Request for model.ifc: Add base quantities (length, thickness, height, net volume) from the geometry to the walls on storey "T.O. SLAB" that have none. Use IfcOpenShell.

First a look at what the model holds.

```python
import ifcopenshell
import ifcopenshell.util.element
import ifcopenshell.util.unit

model = ifcopenshell.open("model.ifc")
print(model.schema)
for unit_type in ("LENGTHUNIT", "AREAUNIT", "VOLUMEUNIT"):
    print(unit_type, ifcopenshell.util.unit.calculate_unit_scale(model, unit_type))
storey = next(s for s in model.by_type("IfcBuildingStorey") if s.Name == "T.O. SLAB")
walls = [e for e in ifcopenshell.util.element.get_decomposition(storey) if e.is_a("IfcWall")]
for e in sorted(walls, key=lambda e: e.id()):
    print(e.id(), e.is_a(), e.Name, list(ifcopenshell.util.element.get_psets(e, qtos_only=True)), sep=" | ")
```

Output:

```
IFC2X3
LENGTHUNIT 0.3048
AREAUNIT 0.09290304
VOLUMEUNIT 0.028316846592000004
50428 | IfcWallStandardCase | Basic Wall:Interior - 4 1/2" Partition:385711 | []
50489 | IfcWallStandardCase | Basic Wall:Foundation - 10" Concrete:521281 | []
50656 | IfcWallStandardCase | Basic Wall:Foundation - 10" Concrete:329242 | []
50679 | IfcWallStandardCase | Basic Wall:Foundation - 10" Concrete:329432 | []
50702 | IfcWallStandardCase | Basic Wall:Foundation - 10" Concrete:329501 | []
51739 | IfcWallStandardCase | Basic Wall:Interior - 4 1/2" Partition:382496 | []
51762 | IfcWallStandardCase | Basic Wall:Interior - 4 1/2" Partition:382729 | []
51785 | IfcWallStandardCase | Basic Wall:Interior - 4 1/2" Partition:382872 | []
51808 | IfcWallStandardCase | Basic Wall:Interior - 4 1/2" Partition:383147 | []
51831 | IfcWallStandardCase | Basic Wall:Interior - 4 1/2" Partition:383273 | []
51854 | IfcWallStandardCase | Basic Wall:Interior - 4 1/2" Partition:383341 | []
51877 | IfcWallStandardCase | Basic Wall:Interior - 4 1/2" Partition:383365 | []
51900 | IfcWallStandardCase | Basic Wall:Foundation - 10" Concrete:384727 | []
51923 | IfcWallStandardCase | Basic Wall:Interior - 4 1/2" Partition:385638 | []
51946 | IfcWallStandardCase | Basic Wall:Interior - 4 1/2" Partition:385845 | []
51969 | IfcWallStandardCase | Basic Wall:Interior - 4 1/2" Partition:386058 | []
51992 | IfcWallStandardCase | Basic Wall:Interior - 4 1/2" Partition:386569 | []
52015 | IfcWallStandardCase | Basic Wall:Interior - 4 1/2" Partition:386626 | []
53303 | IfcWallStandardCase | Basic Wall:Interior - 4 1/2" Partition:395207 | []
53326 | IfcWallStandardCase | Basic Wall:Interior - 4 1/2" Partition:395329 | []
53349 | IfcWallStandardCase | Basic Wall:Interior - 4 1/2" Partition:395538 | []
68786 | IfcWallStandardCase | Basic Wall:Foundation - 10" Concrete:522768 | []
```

```python
import ifcopenshell
import ifcopenshell.api.pset
import ifcopenshell.geom
import ifcopenshell.util.element
import ifcopenshell.util.shape
import ifcopenshell.util.unit

model = ifcopenshell.open("model.ifc")
unit_scale = ifcopenshell.util.unit.calculate_unit_scale(model)
volume_scale = ifcopenshell.util.unit.calculate_unit_scale(model, "VOLUMEUNIT")
settings = ifcopenshell.geom.settings()

storey = next(s for s in model.by_type("IfcBuildingStorey") if s.Name == "T.O. SLAB")
walls = [e for e in ifcopenshell.util.element.get_decomposition(storey) if e.is_a("IfcWall")]

for e in sorted(walls, key=lambda e: e.id()):
    if ifcopenshell.util.element.get_psets(e, qtos_only=True, should_inherit=False):
        continue
    # Geometry comes back in metres, in the element's own axes.
    shape = ifcopenshell.geom.create_shape(settings, e)
    values = {
        "Length": ifcopenshell.util.shape.get_x(shape.geometry) / unit_scale,
        "Width": ifcopenshell.util.shape.get_y(shape.geometry) / unit_scale,
        "Height": ifcopenshell.util.shape.get_z(shape.geometry) / unit_scale,
        "NetVolume": ifcopenshell.util.shape.get_volume(shape.geometry) / volume_scale,
    }
    qto = ifcopenshell.api.pset.add_qto(model, product=e, name="BaseQuantities")
    ifcopenshell.api.pset.edit_qto(model, qto=qto, properties=values)
    print(e.id(), {k: round(v, 3) for k, v in values.items()})

model.write("model_v2.ifc")
```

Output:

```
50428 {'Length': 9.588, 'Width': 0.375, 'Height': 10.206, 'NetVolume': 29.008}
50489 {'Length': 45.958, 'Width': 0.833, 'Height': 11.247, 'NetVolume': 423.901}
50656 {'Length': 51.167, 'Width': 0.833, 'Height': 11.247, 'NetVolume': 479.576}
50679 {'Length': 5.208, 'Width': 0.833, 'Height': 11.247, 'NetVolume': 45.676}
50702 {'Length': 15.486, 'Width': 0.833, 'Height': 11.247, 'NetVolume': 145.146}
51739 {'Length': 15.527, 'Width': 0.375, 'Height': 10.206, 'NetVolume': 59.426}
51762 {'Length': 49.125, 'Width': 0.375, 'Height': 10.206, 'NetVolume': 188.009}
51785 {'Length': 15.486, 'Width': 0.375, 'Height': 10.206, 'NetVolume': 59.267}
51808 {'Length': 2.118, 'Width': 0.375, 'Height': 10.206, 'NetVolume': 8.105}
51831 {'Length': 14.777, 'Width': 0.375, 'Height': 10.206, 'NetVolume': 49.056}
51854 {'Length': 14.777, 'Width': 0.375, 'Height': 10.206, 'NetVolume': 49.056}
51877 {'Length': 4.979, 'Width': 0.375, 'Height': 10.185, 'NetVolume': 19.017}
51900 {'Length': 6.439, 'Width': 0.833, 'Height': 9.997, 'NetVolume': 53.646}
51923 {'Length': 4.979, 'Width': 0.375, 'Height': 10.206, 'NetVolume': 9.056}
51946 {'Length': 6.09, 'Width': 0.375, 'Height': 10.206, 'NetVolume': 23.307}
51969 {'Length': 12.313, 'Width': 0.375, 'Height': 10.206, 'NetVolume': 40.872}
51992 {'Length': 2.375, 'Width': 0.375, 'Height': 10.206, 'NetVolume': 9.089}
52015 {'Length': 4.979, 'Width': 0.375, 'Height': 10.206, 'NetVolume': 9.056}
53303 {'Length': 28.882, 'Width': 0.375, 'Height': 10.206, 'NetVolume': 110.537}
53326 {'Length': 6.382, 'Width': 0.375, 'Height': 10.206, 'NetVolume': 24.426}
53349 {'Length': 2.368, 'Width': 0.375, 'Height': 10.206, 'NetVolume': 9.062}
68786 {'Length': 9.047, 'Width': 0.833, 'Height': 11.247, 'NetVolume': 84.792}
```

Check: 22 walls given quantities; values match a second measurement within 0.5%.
